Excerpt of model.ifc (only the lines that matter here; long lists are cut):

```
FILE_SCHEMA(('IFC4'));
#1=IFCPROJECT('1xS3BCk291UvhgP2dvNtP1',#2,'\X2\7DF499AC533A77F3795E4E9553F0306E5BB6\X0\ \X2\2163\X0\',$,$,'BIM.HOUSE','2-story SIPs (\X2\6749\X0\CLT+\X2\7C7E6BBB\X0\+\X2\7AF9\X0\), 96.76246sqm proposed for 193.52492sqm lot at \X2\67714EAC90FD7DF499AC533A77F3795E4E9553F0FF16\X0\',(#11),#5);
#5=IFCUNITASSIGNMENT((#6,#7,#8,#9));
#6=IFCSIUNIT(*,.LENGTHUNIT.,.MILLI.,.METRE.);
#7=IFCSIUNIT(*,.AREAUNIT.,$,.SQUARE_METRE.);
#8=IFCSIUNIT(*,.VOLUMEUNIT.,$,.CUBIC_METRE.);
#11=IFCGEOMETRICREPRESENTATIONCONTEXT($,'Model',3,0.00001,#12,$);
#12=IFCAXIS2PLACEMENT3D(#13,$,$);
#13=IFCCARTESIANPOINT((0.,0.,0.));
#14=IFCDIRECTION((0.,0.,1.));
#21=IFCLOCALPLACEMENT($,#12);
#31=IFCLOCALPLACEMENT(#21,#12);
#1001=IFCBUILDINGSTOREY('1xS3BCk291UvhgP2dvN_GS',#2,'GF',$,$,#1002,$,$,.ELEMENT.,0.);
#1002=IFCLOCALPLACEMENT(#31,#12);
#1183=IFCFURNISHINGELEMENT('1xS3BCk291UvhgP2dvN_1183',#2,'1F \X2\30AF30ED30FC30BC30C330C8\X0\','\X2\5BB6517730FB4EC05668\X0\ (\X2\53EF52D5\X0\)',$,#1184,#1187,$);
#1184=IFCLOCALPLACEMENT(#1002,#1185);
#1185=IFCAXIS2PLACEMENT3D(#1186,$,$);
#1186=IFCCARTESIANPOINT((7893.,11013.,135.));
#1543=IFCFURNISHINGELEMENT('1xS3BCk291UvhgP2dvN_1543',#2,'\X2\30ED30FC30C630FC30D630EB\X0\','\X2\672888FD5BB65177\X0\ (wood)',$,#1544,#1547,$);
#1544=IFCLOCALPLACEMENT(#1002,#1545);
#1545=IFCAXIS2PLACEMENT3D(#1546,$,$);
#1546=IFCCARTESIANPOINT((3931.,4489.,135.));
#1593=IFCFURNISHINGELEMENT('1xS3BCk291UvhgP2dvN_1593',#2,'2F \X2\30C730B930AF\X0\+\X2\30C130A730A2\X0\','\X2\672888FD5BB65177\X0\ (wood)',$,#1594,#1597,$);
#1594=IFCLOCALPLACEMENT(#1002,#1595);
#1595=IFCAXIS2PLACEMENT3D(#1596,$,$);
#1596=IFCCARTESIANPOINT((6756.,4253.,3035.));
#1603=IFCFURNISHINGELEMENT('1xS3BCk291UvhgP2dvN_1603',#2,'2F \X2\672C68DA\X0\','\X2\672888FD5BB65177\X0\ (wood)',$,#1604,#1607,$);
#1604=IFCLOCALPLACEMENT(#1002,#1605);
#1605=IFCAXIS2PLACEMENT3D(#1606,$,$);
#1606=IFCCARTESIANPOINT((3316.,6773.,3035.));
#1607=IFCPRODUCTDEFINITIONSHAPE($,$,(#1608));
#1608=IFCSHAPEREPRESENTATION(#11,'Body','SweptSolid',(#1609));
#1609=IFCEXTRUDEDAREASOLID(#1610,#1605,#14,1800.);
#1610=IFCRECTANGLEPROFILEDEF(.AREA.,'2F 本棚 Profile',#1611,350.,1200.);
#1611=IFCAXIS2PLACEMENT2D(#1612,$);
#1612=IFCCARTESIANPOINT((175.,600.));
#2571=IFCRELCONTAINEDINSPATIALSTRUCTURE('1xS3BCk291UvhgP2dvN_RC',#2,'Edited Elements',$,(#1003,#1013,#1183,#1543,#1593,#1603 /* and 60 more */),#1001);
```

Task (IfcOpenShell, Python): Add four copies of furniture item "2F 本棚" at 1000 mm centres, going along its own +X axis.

```python
import ifcopenshell
import ifcopenshell.api.geometry
import ifcopenshell.api.root
import ifcopenshell.util.element
import ifcopenshell.util.placement
import ifcopenshell.util.unit

model = ifcopenshell.open("model.ifc")
unit_scale = ifcopenshell.util.unit.calculate_unit_scale(model)


def reuse_history(source, copy):
    """copy_class also copies each property set's owner history, people and application; keep the originals."""
    for rel in copy.IsDefinedBy:
        if rel.is_a("IfcRelDefinesByProperties") and (history := rel.RelatingPropertyDefinition.OwnerHistory):
            rel.RelatingPropertyDefinition.OwnerHistory = source.OwnerHistory
            ifcopenshell.util.element.remove_deep2(model, history)


source = model.by_guid("1xS3BCk291UvhgP2dvN_1603")
base = ifcopenshell.util.placement.get_local_placement(source.ObjectPlacement)
step = base[:3, 0] * 1 / unit_scale

for i in range(1, 5):
    copy = ifcopenshell.api.root.copy_class(model, product=source)
    copy.Representation = ifcopenshell.util.element.copy_deep(
        model, source.Representation, exclude=["IfcGeometricRepresentationContext", "IfcRepresentationMap"]
    )
    reuse_history(source, copy)
    matrix = base.copy()
    matrix[:3, 3] += i * step
    print("added at", matrix[:3, 3].round(3) + 0.0)
    ifcopenshell.api.geometry.edit_object_placement(model, product=copy, matrix=matrix, is_si=False)

model.write("model_rev.ifc")
```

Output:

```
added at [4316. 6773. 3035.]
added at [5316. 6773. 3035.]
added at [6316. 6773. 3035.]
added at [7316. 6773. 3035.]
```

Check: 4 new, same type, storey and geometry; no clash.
